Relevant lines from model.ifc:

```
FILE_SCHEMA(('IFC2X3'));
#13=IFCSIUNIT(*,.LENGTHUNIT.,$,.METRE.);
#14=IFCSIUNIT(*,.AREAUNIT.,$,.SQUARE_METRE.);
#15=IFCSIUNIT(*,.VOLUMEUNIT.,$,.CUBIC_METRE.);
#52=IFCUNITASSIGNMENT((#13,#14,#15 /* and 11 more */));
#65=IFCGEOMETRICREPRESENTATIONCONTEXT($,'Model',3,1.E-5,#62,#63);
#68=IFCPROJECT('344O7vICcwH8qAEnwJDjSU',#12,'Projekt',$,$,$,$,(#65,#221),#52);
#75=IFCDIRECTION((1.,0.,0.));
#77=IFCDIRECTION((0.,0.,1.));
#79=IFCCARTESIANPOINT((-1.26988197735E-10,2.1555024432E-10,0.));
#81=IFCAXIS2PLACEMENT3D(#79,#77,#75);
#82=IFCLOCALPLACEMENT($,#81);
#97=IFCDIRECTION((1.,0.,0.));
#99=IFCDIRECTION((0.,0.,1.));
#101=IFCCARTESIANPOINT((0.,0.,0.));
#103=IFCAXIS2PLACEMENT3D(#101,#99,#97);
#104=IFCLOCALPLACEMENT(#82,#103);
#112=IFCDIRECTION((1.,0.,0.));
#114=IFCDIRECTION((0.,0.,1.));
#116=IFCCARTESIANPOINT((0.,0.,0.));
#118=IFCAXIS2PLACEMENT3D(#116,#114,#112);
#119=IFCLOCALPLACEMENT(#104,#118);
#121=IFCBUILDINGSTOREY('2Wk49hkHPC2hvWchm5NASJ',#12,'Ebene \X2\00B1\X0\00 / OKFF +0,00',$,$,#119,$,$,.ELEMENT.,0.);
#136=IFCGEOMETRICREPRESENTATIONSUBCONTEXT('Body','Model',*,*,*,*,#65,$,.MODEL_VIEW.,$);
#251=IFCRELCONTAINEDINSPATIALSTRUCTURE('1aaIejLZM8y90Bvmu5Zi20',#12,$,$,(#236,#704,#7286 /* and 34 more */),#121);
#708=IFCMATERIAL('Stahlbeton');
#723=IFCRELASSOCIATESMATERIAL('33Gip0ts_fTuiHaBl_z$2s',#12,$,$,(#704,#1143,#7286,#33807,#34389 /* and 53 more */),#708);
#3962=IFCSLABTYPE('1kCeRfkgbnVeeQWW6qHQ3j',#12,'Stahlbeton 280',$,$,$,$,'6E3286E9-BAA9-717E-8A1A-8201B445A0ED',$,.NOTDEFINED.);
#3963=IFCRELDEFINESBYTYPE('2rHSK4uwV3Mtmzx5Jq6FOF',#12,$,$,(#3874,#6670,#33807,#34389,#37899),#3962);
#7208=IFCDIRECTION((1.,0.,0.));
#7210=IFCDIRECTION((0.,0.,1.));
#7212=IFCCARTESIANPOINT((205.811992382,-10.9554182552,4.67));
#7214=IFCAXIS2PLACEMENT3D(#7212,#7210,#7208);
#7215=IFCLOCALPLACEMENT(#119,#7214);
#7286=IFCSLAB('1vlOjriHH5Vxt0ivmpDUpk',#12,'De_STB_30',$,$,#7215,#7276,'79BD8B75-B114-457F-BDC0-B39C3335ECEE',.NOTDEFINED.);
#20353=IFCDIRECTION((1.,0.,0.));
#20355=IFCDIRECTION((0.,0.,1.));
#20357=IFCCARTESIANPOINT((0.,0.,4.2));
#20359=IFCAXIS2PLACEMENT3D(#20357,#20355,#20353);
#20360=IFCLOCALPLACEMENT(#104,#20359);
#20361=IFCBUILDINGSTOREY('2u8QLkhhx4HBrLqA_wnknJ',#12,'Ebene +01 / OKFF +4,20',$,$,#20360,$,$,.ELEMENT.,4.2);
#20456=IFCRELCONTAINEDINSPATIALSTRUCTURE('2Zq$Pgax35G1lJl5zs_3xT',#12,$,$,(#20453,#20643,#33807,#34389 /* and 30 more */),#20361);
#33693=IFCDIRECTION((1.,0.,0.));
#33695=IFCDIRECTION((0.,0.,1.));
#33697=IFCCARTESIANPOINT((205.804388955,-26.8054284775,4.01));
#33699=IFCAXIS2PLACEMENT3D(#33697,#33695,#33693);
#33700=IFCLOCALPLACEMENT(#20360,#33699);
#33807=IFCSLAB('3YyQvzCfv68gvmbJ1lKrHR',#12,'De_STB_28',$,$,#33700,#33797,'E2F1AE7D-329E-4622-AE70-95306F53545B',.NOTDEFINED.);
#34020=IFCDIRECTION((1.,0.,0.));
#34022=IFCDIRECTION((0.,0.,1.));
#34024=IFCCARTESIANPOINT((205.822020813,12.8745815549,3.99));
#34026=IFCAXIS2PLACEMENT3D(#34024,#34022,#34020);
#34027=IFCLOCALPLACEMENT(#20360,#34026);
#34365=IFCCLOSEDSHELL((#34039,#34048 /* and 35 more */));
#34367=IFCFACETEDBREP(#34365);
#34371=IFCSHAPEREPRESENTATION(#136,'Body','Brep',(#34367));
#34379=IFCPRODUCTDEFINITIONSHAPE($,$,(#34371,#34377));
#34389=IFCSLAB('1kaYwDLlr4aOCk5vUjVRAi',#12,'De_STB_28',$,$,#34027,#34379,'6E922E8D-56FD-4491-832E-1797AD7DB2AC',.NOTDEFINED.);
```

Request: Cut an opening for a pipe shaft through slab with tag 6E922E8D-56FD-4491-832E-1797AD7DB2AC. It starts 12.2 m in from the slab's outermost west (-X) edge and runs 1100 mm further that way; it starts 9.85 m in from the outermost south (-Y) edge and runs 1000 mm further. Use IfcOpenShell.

```python
import numpy as np
import ifcopenshell
import ifcopenshell.api.feature
import ifcopenshell.api.geometry
import ifcopenshell.api.root
import ifcopenshell.geom
import ifcopenshell.util.placement
import ifcopenshell.util.representation
import ifcopenshell.util.shape
import ifcopenshell.util.unit

model = ifcopenshell.open("model.ifc")
unit_scale = ifcopenshell.util.unit.calculate_unit_scale(model)
settings = ifcopenshell.geom.settings()


def volume(element):
    """Net volume in cubic metres, openings subtracted."""
    shape = ifcopenshell.geom.create_shape(settings, element)
    return ifcopenshell.util.shape.get_volume(shape.geometry)


slab = model.by_id(34389)
before = volume(slab)

# Extent in the slab's own axes, in metres. The edges named are its -X and -Y sides.
slab_shape = ifcopenshell.geom.create_shape(settings, slab)
vertices = ifcopenshell.util.shape.get_vertices(slab_shape.geometry)
x_min, y_min, bottom = vertices.min(axis=0)
top = vertices[:, 2].max()

opening = ifcopenshell.api.root.create_entity(model, ifc_class="IfcOpeningElement", name="Pipe shaft opening")
context = ifcopenshell.util.representation.get_context(model, "Model", "Body", "MODEL_VIEW")
width, depth = 1.1, 1
outline = [(0.0, 0.0), (width, 0.0), (width, depth), (0.0, depth), (0.0, 0.0)]
# Overshoot both faces by 50 mm so the cut is clean.
shape = ifcopenshell.api.geometry.add_slab_representation(
    model, context=context, depth=top - bottom + 0.1, polyline=outline
)
ifcopenshell.api.geometry.assign_representation(model, product=opening, representation=shape)

matrix = ifcopenshell.util.placement.get_local_placement(slab.ObjectPlacement)
matrix[:, 3] = matrix @ np.append(np.array([x_min + 12.2, y_min + 9.85, bottom - 0.05]) / unit_scale, 1.0)
ifcopenshell.api.geometry.edit_object_placement(model, product=opening, matrix=matrix, is_si=False)
ifcopenshell.api.feature.add_feature(model, feature=opening, element=slab)

after = volume(slab)

print(f"slab volume {before:.3f} -> {after:.3f} m3")

model.write("model_updated.ifc")
```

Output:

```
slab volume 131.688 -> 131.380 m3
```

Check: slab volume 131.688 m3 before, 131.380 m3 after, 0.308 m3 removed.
